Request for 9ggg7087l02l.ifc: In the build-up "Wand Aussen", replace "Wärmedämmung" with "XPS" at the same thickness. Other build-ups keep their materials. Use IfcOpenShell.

First a look at what the model holds.

```python
import ifcopenshell
import ifcopenshell.util.element

model = ifcopenshell.open("9ggg7087l02l.ifc")
print(model.schema)
for layer_set in model.by_type("IfcMaterialLayerSet"):
    if layer_set.LayerSetName == "Wand Aussen":
        for layer in layer_set.MaterialLayers:
            print(layer.id(), layer.Material and layer.Material.Name, layer.LayerThickness, sep=" | ")
        print(len(ifcopenshell.util.element.get_elements_by_material(model, layer_set)), "elements and types use it")
print(sorted(m.Name for m in model.by_type("IfcMaterial") if m.Name)[:60])
```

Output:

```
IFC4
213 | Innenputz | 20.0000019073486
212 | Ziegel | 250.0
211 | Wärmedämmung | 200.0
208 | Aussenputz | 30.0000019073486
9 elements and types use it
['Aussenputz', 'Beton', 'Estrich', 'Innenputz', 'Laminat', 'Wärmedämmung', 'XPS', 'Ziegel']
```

```python
import ifcopenshell
import ifcopenshell.api.material

model = ifcopenshell.open("9ggg7087l02l.ifc")

layer_set = next(s for s in model.by_type("IfcMaterialLayerSet") if s.LayerSetName == "Wand Aussen")
layer = next(l for l in layer_set.MaterialLayers if l.Material and l.Material.Name == "Wärmedämmung")
material = next(m for m in model.by_type("IfcMaterial") if m.Name == "XPS")

# Point this one layer at the other material; renaming the old one would change it everywhere.
ifcopenshell.api.material.edit_layer(model, layer=layer, attributes={}, material=material)

print([l.Material.Name if l.Material else None for l in layer_set.MaterialLayers])

model.write("9ggg7087l02l_v2.ifc")
```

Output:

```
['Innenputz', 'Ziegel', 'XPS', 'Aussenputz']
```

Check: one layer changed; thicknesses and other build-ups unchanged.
